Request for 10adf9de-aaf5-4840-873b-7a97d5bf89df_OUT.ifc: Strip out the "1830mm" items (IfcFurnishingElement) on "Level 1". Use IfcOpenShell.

First a look at what the model holds.

```python
import ifcopenshell
import ifcopenshell.util.element

model = ifcopenshell.open("10adf9de-aaf5-4840-873b-7a97d5bf89df_OUT.ifc")
print(model.schema)
storey = next(s for s in model.by_type("IfcBuildingStorey") if s.Name == "Level 1")
furniture = [e for e in ifcopenshell.util.element.get_decomposition(storey) if e.is_a("IfcFurnishingElement")]
seen = {}
for e in furniture:
    element_type = ifcopenshell.util.element.get_type(e)
    name = element_type.Name if element_type not in (None, e) else None
    seen[name] = seen.get(name, 0) + 1
for name, count in sorted(seen.items(), key=str):
    print(count, "x", name)
```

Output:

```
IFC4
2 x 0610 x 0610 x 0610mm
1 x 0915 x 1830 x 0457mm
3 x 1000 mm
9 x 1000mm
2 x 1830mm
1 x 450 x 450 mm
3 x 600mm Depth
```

```python
import ifcopenshell
import ifcopenshell.api.root
import ifcopenshell.util.element

model = ifcopenshell.open("10adf9de-aaf5-4840-873b-7a97d5bf89df_OUT.ifc")

storey = next(s for s in model.by_type("IfcBuildingStorey") if s.Name == "Level 1")
furniture = [e for e in ifcopenshell.util.element.get_decomposition(storey) if e.is_a("IfcFurnishingElement")]
targets = [e for e in furniture if (t := ifcopenshell.util.element.get_type(e)) not in (None, e) and t.Name == "1830mm"]

for e in targets:
    ifcopenshell.api.root.remove_product(model, product=e)
print(len(targets), "removed")

model.write("10adf9de-aaf5-4840-873b-7a97d5bf89df_OUT_updated.ifc")
```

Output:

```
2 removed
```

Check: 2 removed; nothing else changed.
